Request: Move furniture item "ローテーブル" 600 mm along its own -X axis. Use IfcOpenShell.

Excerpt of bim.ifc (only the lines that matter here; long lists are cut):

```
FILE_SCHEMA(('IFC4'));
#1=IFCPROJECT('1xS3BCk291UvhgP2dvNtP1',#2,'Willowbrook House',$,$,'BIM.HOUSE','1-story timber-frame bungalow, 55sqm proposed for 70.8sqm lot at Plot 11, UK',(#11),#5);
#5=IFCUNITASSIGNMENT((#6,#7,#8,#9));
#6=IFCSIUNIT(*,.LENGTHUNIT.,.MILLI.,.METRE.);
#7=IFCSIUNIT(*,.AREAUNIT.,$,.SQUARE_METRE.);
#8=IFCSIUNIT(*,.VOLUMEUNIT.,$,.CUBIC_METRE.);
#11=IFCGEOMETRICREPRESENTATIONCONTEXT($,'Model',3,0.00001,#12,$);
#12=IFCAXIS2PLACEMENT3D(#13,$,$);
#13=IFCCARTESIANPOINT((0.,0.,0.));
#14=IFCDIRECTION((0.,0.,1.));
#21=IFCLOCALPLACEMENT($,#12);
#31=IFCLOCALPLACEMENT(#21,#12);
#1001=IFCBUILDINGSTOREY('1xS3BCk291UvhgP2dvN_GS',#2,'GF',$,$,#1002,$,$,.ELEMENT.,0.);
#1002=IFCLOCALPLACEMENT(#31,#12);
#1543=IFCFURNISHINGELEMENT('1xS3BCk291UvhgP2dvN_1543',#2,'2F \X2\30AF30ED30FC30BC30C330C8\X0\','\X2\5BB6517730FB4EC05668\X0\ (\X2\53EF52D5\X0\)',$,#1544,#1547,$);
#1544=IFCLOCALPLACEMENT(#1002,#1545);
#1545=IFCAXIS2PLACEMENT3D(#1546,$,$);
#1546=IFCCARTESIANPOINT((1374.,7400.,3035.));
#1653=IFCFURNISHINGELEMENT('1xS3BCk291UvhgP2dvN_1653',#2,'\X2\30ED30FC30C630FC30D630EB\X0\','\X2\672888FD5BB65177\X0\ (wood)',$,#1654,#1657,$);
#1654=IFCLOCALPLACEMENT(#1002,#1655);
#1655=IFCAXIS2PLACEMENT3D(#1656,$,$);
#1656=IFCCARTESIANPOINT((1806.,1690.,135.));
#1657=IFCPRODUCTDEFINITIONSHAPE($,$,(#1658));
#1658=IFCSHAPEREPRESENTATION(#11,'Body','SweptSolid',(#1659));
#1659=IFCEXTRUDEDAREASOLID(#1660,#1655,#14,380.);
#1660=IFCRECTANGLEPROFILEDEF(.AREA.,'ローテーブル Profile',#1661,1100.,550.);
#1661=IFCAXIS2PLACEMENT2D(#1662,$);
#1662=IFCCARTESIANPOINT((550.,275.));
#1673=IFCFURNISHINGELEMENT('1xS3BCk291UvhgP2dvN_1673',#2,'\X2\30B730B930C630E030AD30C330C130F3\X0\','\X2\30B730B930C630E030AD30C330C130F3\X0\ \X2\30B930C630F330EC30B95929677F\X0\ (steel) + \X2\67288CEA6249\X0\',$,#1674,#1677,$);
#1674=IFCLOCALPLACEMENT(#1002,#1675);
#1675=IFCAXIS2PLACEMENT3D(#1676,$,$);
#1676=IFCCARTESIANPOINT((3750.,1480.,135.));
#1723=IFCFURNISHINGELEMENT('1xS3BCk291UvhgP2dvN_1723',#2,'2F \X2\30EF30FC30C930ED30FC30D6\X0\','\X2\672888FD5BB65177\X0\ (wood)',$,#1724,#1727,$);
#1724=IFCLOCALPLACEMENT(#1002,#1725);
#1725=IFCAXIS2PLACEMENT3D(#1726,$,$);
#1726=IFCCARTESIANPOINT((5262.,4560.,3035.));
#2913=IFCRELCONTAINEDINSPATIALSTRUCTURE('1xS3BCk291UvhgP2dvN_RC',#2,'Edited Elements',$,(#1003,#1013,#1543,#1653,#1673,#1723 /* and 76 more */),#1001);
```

```python
import ifcopenshell
import ifcopenshell.api.geometry
import ifcopenshell.util.placement
import ifcopenshell.util.unit

model = ifcopenshell.open("bim.ifc")
unit_scale = ifcopenshell.util.unit.calculate_unit_scale(model)

item = model.by_id(1653)
matrix = ifcopenshell.util.placement.get_local_placement(item.ObjectPlacement)
matrix[:3, 3] -= matrix[:3, 0] * 0.6 / unit_scale
ifcopenshell.api.geometry.edit_object_placement(model, product=item, matrix=matrix, is_si=False)

print(ifcopenshell.util.placement.get_local_placement(item.ObjectPlacement).round(3) + 0.0)

model.write("bim_v2.ifc")
```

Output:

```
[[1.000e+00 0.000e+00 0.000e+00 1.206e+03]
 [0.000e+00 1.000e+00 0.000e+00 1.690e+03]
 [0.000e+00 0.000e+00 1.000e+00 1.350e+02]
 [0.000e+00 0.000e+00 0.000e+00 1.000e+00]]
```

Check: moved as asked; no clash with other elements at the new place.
